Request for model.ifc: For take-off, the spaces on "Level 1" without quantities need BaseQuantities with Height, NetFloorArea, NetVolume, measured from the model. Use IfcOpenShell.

First a look at what the model holds.

```python
import ifcopenshell
import ifcopenshell.util.element
import ifcopenshell.util.unit

model = ifcopenshell.open("model.ifc")
print(model.schema)
for unit_type in ("LENGTHUNIT", "AREAUNIT", "VOLUMEUNIT"):
    print(unit_type, ifcopenshell.util.unit.calculate_unit_scale(model, unit_type))
storey = next(s for s in model.by_type("IfcBuildingStorey") if s.Name == "Level 1")
spaces = [e for e in ifcopenshell.util.element.get_decomposition(storey) if e.is_a("IfcSpace")]
for e in sorted(spaces, key=lambda e: e.id()):
    print(e.id(), e.is_a(), e.Name, list(ifcopenshell.util.element.get_psets(e, qtos_only=True)), sep=" | ")
```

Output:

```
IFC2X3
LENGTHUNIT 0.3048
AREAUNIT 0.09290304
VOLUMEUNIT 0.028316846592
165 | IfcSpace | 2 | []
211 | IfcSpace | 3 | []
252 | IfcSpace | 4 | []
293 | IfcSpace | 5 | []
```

```python
import ifcopenshell
import ifcopenshell.api.pset
import ifcopenshell.geom
import ifcopenshell.util.element
import ifcopenshell.util.shape
import ifcopenshell.util.unit

model = ifcopenshell.open("model.ifc")
unit_scale = ifcopenshell.util.unit.calculate_unit_scale(model)
area_scale = ifcopenshell.util.unit.calculate_unit_scale(model, "AREAUNIT")
volume_scale = ifcopenshell.util.unit.calculate_unit_scale(model, "VOLUMEUNIT")
settings = ifcopenshell.geom.settings()

storey = next(s for s in model.by_type("IfcBuildingStorey") if s.Name == "Level 1")
spaces = [e for e in ifcopenshell.util.element.get_decomposition(storey) if e.is_a("IfcSpace")]

for e in sorted(spaces, key=lambda e: e.id()):
    if ifcopenshell.util.element.get_psets(e, qtos_only=True, should_inherit=False):
        continue
    # Geometry comes back in metres, in the element's own axes.
    shape = ifcopenshell.geom.create_shape(settings, e)
    values = {
        "Height": ifcopenshell.util.shape.get_z(shape.geometry) / unit_scale,
        "NetFloorArea": ifcopenshell.util.shape.get_footprint_area(shape.geometry) / area_scale,
        "NetVolume": ifcopenshell.util.shape.get_volume(shape.geometry) / volume_scale,
    }
    qto = ifcopenshell.api.pset.add_qto(model, product=e, name="BaseQuantities")
    ifcopenshell.api.pset.edit_qto(model, qto=qto, properties=values)
    print(e.id(), {k: round(v, 3) for k, v in values.items()})

model.write("model_updated.ifc")
```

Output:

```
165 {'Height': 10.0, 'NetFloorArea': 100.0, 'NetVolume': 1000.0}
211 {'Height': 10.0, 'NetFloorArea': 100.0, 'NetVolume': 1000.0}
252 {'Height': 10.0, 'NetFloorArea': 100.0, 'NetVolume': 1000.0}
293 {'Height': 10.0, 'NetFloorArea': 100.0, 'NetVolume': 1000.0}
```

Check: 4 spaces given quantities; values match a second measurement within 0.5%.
